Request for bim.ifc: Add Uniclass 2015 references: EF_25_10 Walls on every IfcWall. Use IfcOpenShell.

First a look at what the model holds.

```python
import ifcopenshell

model = ifcopenshell.open("bim.ifc")
print(model.schema)
print("classifications:", [c.Name for c in model.by_type("IfcClassification")])
for ifc_class in ("IfcDoor", "IfcRoof", "IfcStair", "IfcWall", "IfcWindow"):
    print(ifc_class, len(model.by_type(ifc_class)))
```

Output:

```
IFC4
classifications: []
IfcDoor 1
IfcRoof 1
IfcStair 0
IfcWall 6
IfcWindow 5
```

```python
import ifcopenshell
import ifcopenshell.api.classification

model = ifcopenshell.open("bim.ifc")

system = ifcopenshell.api.classification.add_classification(model, classification="Uniclass 2015")

codes = {
    "IfcWall": ("EF_25_10", "Walls"),
}
for ifc_class, (code, name) in codes.items():
    products = model.by_type(ifc_class)
    ifcopenshell.api.classification.add_reference(
        model, products=products, classification=system, identification=code, name=name
    )
    print(code, len(products))

model.write("bim_v2.ifc")
```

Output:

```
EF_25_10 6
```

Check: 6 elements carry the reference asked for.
